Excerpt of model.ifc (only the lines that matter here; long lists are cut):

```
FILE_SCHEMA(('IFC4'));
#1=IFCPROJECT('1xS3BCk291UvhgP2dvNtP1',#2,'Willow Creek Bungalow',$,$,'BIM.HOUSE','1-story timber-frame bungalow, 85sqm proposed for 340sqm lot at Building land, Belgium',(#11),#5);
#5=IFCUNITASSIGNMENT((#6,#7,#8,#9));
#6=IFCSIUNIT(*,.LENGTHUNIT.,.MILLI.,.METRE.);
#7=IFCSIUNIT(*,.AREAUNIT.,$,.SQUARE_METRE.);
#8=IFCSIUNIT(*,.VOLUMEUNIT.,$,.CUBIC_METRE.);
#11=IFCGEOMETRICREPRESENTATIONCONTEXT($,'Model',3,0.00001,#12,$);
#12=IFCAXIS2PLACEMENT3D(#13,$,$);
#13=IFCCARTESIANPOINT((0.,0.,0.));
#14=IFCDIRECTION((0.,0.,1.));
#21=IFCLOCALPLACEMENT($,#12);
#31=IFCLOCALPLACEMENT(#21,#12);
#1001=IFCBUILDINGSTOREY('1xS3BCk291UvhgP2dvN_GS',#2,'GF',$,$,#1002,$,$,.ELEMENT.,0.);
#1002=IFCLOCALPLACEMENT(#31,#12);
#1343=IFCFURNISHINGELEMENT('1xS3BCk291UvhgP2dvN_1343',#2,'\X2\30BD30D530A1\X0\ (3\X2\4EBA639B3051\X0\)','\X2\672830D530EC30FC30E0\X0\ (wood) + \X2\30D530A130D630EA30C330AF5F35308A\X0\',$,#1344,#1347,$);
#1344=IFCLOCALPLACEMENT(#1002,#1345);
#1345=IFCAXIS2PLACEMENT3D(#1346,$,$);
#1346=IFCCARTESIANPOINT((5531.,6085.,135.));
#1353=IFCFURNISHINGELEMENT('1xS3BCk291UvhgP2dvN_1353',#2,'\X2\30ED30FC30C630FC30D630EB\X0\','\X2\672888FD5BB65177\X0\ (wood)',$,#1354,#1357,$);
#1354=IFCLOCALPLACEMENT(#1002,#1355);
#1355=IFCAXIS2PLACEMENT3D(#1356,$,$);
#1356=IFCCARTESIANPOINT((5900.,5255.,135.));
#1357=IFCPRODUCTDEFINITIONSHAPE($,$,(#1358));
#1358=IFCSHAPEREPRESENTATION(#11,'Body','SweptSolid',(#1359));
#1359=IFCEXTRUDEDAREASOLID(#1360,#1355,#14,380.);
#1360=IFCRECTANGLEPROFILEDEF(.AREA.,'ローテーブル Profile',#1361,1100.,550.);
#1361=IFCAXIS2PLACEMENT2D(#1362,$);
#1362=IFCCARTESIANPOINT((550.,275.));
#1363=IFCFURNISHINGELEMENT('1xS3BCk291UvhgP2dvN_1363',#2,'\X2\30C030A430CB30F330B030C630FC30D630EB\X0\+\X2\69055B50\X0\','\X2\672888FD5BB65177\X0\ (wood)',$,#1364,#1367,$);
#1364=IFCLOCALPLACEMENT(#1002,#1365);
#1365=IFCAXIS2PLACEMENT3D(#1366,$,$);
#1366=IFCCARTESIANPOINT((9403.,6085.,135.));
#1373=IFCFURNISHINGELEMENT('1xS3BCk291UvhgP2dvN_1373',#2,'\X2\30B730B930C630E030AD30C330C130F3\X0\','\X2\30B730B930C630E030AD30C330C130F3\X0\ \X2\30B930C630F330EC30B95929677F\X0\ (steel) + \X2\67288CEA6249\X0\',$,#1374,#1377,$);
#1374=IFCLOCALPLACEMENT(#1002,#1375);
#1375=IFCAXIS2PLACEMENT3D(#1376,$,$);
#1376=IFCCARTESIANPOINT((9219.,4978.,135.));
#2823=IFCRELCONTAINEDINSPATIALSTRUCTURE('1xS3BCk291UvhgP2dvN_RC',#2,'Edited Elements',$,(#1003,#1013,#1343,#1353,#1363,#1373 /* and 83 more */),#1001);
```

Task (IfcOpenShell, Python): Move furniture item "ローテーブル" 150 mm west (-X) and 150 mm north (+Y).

```python
import ifcopenshell
import ifcopenshell.api.geometry
import ifcopenshell.util.placement
import ifcopenshell.util.unit

model = ifcopenshell.open("model.ifc")
unit_scale = ifcopenshell.util.unit.calculate_unit_scale(model)

item = model.by_id(1353)
matrix = ifcopenshell.util.placement.get_local_placement(item.ObjectPlacement)
matrix[0, 3] -= 0.15 / unit_scale
matrix[1, 3] += 0.15 / unit_scale
ifcopenshell.api.geometry.edit_object_placement(model, product=item, matrix=matrix, is_si=False)

print(ifcopenshell.util.placement.get_local_placement(item.ObjectPlacement).round(3) + 0.0)

model.write("model_rev.ifc")
```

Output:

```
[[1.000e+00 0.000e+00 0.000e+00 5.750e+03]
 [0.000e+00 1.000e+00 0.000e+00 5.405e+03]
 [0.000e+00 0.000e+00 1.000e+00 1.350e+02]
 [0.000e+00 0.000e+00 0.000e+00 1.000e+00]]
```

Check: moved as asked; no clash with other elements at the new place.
